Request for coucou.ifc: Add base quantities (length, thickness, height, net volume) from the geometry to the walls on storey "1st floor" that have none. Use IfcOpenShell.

First a look at what the model holds.

```python
import ifcopenshell
import ifcopenshell.util.element
import ifcopenshell.util.unit

model = ifcopenshell.open("coucou.ifc")
print(model.schema)
for unit_type in ("LENGTHUNIT", "AREAUNIT", "VOLUMEUNIT"):
    print(unit_type, ifcopenshell.util.unit.calculate_unit_scale(model, unit_type))
storey = next(s for s in model.by_type("IfcBuildingStorey") if s.Name == "1st floor")
walls = [e for e in ifcopenshell.util.element.get_decomposition(storey) if e.is_a("IfcWall")]
for e in sorted(walls, key=lambda e: e.id()):
    print(e.id(), e.is_a(), e.Name, list(ifcopenshell.util.element.get_psets(e, qtos_only=True)), sep=" | ")
```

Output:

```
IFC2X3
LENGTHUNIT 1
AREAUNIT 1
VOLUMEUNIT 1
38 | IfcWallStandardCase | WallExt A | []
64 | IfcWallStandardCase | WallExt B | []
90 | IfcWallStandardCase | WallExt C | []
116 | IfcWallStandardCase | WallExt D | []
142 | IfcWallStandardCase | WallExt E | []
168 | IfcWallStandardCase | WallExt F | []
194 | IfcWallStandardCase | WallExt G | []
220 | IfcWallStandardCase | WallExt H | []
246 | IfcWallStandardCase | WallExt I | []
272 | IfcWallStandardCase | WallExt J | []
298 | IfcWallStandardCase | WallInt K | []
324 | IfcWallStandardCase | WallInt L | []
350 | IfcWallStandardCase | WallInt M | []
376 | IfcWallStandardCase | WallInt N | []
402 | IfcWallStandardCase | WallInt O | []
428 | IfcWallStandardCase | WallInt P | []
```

```python
import ifcopenshell
import ifcopenshell.api.pset
import ifcopenshell.geom
import ifcopenshell.util.element
import ifcopenshell.util.shape
import ifcopenshell.util.unit

model = ifcopenshell.open("coucou.ifc")
unit_scale = ifcopenshell.util.unit.calculate_unit_scale(model)
volume_scale = ifcopenshell.util.unit.calculate_unit_scale(model, "VOLUMEUNIT")
settings = ifcopenshell.geom.settings()

storey = next(s for s in model.by_type("IfcBuildingStorey") if s.Name == "1st floor")
walls = [e for e in ifcopenshell.util.element.get_decomposition(storey) if e.is_a("IfcWall")]

for e in sorted(walls, key=lambda e: e.id()):
    if ifcopenshell.util.element.get_psets(e, qtos_only=True, should_inherit=False):
        continue
    # Geometry comes back in metres, in the element's own axes.
    shape = ifcopenshell.geom.create_shape(settings, e)
    values = {
        "Length": ifcopenshell.util.shape.get_x(shape.geometry) / unit_scale,
        "Width": ifcopenshell.util.shape.get_y(shape.geometry) / unit_scale,
        "Height": ifcopenshell.util.shape.get_z(shape.geometry) / unit_scale,
        "NetVolume": ifcopenshell.util.shape.get_volume(shape.geometry) / volume_scale,
    }
    qto = ifcopenshell.api.pset.add_qto(model, product=e, name="BaseQuantities")
    ifcopenshell.api.pset.edit_qto(model, qto=qto, properties=values)
    print(e.id(), {k: round(v, 3) for k, v in values.items()})

model.write("coucou-out.ifc")
```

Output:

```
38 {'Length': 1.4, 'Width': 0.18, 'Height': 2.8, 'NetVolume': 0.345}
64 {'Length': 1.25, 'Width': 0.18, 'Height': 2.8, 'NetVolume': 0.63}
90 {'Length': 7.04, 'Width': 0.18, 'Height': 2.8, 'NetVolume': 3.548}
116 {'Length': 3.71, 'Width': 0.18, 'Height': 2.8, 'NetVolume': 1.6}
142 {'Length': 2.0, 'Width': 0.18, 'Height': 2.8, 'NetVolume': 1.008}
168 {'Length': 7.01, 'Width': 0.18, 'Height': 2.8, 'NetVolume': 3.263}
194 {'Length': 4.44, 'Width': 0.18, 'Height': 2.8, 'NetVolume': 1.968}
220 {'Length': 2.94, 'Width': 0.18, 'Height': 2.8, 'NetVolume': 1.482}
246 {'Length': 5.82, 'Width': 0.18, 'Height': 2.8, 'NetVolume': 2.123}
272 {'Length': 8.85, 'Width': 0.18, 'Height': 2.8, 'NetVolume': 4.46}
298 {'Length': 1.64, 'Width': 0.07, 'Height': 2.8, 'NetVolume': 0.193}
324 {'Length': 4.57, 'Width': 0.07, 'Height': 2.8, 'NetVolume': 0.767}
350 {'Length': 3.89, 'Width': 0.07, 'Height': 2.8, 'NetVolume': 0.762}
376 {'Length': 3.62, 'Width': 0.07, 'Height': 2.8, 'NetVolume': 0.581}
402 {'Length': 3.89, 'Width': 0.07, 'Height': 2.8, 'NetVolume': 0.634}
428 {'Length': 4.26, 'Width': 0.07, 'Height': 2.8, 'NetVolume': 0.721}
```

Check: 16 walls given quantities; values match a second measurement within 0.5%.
